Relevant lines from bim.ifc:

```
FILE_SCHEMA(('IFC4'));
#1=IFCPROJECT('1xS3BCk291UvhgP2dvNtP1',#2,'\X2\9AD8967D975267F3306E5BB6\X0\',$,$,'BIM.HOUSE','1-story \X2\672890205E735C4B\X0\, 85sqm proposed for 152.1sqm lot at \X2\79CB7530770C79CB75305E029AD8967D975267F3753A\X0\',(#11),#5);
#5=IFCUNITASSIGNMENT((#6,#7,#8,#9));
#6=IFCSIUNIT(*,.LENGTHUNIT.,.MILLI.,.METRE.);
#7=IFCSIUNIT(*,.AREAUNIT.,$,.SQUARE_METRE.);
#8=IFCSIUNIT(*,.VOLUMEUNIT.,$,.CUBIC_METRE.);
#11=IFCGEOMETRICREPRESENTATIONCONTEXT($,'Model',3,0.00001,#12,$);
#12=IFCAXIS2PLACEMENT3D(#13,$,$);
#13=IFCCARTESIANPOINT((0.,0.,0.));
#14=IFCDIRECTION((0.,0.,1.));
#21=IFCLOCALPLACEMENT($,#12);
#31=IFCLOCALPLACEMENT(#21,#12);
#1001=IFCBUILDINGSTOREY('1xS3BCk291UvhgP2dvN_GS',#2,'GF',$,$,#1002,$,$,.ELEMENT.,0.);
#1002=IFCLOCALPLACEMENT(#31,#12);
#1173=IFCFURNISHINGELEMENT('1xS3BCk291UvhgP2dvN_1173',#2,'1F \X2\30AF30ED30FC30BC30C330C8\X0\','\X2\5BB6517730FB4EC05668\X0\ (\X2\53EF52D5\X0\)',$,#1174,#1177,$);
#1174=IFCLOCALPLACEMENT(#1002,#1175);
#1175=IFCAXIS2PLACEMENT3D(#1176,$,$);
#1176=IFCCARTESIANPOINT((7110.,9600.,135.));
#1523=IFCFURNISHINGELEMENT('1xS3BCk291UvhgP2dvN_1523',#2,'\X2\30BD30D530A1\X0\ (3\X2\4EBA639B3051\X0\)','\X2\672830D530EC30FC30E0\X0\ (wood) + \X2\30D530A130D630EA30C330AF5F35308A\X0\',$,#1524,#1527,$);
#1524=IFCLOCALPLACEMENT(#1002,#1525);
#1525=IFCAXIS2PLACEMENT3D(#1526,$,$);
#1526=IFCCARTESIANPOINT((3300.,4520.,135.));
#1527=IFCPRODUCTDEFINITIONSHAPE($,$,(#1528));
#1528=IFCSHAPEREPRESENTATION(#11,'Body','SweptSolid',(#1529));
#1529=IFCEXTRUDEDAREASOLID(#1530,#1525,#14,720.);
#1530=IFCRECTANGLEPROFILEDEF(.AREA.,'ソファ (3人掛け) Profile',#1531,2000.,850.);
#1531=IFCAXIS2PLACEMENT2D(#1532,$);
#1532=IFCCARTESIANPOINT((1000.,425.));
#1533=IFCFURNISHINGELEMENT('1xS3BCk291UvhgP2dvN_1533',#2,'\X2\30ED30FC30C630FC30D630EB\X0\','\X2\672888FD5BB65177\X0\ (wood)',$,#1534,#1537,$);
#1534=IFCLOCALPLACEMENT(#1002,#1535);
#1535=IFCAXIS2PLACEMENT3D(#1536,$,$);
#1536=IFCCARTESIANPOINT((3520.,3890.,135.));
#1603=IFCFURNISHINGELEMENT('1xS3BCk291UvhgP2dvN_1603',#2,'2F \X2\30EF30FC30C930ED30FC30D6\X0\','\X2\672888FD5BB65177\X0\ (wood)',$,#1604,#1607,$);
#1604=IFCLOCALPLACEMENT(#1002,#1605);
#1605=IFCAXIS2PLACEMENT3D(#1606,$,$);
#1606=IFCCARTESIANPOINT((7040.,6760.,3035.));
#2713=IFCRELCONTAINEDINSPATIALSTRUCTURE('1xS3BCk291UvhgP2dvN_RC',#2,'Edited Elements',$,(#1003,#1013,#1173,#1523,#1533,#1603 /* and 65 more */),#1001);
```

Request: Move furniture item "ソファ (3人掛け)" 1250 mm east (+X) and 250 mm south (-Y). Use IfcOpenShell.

```python
import ifcopenshell
import ifcopenshell.api.geometry
import ifcopenshell.util.placement

model = ifcopenshell.open("bim.ifc")

item = model.by_id(1523)
matrix = ifcopenshell.util.placement.get_local_placement(item.ObjectPlacement)
matrix[0, 3] += 1250.0
matrix[1, 3] -= 250.0
ifcopenshell.api.geometry.edit_object_placement(model, product=item, matrix=matrix, is_si=False)

print(ifcopenshell.util.placement.get_local_placement(item.ObjectPlacement).round(3) + 0.0)

model.write("bim_edited.ifc")
```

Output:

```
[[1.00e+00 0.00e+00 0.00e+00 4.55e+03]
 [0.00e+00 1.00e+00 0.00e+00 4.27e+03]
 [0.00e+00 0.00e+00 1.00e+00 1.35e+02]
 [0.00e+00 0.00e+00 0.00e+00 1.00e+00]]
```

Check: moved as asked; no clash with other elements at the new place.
